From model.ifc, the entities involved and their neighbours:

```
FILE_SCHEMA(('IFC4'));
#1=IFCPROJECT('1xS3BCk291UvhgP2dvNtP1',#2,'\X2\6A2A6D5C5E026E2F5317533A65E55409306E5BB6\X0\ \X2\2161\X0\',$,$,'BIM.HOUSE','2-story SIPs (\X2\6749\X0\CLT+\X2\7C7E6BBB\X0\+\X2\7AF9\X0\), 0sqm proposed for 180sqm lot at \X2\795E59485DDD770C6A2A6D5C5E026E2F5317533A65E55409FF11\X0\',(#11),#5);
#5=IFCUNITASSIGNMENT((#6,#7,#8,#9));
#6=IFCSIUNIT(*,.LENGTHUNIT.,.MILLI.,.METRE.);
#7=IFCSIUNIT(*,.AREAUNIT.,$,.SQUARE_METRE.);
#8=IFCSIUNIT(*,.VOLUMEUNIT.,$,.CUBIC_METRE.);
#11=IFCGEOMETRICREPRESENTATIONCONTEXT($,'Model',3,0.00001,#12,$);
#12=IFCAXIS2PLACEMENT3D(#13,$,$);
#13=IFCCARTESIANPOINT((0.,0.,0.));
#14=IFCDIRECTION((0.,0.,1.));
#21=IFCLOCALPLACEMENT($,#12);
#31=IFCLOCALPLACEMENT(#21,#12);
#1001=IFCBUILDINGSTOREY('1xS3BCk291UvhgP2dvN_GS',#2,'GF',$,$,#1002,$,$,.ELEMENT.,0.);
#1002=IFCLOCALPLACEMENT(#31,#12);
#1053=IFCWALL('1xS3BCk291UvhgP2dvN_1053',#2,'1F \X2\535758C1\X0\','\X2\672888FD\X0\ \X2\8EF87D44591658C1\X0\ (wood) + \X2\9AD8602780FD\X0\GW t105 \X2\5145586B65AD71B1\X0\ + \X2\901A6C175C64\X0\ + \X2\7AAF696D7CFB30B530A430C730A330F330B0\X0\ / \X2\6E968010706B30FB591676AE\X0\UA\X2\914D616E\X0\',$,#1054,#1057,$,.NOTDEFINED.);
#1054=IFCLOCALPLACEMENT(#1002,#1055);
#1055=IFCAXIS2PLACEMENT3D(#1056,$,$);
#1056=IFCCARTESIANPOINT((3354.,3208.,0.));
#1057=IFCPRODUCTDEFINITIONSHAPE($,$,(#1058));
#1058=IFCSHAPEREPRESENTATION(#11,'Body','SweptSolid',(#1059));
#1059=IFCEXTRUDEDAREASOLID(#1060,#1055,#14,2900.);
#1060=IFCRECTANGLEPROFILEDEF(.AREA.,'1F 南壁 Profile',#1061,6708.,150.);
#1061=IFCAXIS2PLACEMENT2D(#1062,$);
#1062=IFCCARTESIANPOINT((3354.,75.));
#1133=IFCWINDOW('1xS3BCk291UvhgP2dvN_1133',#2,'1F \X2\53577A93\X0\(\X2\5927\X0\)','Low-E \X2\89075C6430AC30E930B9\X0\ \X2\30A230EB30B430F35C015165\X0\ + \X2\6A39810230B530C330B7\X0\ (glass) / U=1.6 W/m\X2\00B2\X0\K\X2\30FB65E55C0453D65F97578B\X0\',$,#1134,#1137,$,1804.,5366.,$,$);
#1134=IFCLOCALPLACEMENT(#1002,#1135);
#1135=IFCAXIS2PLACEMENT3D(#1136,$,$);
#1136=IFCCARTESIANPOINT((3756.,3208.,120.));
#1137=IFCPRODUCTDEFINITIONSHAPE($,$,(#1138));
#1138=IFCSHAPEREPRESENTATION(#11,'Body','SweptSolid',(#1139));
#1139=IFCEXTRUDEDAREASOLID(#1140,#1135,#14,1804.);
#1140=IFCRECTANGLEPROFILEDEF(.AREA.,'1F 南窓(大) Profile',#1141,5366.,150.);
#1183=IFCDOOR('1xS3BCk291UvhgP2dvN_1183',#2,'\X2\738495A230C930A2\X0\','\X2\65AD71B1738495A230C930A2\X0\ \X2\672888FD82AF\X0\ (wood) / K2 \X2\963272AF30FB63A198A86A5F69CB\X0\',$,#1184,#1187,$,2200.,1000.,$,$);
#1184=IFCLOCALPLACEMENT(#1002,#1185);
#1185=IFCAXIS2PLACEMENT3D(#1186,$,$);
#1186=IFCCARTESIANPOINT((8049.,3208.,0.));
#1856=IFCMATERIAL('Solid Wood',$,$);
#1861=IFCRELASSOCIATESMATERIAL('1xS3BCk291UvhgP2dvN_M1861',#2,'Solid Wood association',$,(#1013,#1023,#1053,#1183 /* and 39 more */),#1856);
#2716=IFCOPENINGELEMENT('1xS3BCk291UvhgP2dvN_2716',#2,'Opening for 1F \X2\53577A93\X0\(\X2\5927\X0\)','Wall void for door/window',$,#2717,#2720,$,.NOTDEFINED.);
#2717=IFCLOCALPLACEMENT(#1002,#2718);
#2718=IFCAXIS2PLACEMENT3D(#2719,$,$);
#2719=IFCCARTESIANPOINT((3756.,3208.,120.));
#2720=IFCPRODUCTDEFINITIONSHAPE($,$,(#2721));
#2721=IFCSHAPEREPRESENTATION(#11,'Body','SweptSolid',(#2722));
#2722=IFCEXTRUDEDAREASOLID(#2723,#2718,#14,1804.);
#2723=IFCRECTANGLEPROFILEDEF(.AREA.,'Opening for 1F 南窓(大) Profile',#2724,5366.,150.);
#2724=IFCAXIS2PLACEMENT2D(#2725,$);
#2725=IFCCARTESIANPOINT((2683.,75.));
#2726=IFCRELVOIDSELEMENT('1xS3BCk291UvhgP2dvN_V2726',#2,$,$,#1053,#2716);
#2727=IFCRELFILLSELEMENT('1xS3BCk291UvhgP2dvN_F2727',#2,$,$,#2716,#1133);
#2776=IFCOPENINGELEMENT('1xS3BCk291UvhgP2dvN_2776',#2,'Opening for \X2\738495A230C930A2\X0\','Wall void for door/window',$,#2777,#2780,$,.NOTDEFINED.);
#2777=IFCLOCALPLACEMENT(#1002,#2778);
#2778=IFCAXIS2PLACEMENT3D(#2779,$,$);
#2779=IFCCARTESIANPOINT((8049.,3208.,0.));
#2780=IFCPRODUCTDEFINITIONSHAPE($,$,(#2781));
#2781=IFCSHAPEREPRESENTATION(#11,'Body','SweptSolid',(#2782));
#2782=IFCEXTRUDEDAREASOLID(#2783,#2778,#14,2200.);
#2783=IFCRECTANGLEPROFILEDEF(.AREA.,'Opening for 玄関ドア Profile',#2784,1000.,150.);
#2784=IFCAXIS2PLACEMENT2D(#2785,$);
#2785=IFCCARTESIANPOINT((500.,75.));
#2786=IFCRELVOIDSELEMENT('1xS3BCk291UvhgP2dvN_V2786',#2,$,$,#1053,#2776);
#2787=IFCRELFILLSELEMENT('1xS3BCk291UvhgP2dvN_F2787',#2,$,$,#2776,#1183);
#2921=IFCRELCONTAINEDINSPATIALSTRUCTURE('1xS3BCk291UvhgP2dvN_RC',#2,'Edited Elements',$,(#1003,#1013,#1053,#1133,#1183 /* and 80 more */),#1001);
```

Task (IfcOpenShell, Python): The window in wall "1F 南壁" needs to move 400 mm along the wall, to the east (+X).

```python
import ifcopenshell
import ifcopenshell.api.geometry
import ifcopenshell.util.placement

model = ifcopenshell.open("model.ifc")

window = model.by_guid("1xS3BCk291UvhgP2dvN_1133")
opening = window.FillsVoids[0].RelatingOpeningElement
wall = opening.VoidsElements[0].RelatingBuildingElement

wall_matrix = ifcopenshell.util.placement.get_local_placement(wall.ObjectPlacement)
shift = wall_matrix[:3, 0] * 400.0
before = ifcopenshell.util.placement.get_local_placement(window.ObjectPlacement)[:3, 3].copy()

# The window is not placed relative to its opening, so move both.
for product in (opening, window):
    matrix = ifcopenshell.util.placement.get_local_placement(product.ObjectPlacement)
    matrix[:3, 3] += shift
    ifcopenshell.api.geometry.edit_object_placement(model, product=product, matrix=matrix, is_si=False)

after = ifcopenshell.util.placement.get_local_placement(window.ObjectPlacement)[:3, 3]
print("window moved by", (after - before).round(3) + 0.0)

model.write("model_edited.ifc")
```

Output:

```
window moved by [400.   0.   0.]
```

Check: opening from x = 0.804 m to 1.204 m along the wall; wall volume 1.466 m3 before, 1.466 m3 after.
